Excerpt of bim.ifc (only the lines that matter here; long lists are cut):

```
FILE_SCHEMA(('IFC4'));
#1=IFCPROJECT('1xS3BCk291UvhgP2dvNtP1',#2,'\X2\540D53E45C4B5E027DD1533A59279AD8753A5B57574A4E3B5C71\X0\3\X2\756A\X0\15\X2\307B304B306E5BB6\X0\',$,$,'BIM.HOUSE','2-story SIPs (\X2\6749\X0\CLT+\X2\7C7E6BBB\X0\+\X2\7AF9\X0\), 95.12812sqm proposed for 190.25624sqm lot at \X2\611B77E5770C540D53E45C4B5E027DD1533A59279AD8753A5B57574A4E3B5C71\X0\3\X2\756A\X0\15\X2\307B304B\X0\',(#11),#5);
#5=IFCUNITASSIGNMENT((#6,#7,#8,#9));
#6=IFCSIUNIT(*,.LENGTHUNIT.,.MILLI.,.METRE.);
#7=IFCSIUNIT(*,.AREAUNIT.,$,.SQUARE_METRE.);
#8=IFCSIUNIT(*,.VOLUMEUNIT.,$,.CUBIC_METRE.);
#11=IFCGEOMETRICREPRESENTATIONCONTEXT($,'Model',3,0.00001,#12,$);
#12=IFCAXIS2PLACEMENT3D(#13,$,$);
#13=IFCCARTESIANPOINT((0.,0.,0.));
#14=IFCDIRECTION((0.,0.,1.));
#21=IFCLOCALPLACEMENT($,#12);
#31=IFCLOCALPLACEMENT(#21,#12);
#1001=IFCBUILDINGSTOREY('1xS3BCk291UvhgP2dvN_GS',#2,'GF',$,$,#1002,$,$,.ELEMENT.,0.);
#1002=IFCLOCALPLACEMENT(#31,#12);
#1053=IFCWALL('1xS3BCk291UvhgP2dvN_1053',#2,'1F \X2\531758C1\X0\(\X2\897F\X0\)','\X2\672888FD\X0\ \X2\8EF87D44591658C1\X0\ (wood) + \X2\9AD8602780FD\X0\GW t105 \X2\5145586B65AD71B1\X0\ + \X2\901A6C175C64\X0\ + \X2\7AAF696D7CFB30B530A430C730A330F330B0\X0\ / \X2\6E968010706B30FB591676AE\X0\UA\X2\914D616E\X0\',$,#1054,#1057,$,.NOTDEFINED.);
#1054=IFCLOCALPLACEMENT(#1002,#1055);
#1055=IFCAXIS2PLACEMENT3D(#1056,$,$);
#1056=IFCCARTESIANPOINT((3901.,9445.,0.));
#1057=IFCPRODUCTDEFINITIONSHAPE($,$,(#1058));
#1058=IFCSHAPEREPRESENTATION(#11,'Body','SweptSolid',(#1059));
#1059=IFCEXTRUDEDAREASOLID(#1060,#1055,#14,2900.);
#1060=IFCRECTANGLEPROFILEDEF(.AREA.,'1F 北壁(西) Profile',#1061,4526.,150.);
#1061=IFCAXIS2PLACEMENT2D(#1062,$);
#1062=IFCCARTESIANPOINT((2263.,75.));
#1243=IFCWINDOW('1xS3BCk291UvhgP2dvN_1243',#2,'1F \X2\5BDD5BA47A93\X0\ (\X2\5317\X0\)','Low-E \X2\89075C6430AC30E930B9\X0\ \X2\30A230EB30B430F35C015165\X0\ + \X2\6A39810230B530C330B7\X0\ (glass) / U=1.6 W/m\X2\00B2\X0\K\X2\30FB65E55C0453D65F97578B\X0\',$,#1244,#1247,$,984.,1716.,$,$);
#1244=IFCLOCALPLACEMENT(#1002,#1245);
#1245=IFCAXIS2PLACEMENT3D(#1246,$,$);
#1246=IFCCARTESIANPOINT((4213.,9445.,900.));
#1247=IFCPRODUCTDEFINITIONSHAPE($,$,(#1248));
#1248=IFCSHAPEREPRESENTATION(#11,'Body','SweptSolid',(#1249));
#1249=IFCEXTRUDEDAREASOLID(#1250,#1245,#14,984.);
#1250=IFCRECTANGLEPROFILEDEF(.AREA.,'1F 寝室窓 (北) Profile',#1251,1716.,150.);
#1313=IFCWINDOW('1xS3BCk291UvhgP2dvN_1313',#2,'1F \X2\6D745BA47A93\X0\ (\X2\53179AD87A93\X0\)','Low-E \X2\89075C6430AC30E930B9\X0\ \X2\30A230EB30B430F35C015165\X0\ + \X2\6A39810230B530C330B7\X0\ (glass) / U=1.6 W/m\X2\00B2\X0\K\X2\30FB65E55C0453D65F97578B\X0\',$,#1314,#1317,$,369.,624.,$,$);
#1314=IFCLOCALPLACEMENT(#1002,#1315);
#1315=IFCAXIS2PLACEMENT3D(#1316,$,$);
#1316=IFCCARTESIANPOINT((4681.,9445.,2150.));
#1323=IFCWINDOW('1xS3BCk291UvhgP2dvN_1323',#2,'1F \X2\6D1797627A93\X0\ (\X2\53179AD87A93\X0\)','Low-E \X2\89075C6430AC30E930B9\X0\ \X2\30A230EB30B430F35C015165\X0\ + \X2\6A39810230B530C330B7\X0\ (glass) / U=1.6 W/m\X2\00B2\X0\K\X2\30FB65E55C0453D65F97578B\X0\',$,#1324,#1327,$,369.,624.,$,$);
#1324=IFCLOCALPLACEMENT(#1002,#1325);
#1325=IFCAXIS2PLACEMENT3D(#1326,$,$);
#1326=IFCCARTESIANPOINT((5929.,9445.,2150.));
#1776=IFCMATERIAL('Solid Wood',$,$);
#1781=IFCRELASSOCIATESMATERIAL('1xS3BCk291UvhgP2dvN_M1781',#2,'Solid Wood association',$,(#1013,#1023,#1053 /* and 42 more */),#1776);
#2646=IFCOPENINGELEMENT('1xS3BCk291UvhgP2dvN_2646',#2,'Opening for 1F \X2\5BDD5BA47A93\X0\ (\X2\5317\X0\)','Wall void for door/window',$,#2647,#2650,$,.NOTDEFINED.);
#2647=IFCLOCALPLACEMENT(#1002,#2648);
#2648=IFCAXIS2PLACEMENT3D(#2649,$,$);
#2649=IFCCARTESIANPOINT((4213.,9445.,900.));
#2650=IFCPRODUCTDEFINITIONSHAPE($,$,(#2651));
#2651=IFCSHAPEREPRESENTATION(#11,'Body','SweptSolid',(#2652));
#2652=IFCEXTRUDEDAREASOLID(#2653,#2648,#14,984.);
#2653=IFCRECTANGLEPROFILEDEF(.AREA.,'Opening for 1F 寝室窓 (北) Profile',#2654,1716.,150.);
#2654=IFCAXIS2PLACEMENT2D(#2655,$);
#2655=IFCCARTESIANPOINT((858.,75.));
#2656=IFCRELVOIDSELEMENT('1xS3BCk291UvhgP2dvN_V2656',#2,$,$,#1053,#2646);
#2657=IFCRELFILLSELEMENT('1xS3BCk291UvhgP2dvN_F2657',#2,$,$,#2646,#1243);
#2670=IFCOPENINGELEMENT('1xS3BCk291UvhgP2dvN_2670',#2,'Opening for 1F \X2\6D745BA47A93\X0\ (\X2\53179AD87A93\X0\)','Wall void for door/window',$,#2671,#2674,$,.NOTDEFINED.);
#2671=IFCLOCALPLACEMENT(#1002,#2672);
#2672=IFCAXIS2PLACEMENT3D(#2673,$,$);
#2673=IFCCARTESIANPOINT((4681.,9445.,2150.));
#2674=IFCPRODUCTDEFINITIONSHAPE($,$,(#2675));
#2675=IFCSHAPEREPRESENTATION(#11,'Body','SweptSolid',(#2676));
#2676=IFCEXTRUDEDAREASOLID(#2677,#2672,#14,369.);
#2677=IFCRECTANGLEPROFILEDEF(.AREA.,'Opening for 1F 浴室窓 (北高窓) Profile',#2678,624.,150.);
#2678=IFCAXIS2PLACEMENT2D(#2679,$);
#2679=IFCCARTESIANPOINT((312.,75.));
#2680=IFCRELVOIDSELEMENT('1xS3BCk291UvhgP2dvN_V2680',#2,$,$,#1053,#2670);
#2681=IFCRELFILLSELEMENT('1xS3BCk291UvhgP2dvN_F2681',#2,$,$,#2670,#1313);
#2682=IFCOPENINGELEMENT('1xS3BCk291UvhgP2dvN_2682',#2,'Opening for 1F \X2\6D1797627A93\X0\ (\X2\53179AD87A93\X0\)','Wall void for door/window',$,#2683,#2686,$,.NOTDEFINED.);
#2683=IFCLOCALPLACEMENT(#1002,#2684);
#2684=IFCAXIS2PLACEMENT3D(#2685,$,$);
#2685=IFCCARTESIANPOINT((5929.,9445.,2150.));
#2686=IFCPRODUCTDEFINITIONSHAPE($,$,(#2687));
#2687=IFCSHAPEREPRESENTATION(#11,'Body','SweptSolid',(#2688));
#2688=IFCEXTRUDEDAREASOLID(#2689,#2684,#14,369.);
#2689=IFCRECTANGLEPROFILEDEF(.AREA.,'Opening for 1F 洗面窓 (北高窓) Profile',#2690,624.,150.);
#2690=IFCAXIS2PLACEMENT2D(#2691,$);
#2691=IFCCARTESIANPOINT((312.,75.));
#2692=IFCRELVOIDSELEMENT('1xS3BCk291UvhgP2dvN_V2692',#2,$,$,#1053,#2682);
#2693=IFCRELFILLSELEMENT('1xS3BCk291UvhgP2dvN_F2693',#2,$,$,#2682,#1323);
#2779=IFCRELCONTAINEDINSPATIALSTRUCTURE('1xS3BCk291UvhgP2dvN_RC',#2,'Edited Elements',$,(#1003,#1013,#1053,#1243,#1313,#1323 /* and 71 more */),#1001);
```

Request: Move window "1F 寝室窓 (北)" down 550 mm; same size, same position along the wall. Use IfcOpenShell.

```python
import numpy as np
import ifcopenshell
import ifcopenshell.api.geometry
import ifcopenshell.util.placement
import ifcopenshell.util.unit

model = ifcopenshell.open("bim.ifc")
unit_scale = ifcopenshell.util.unit.calculate_unit_scale(model)

window = model.by_guid("1xS3BCk291UvhgP2dvN_1243")
opening = window.FillsVoids[0].RelatingOpeningElement
dz = -0.55 / unit_scale

shift = np.array([0.0, 0.0, dz])
# The window is not placed relative to its opening, so move both.
for product in (opening, window):
    matrix = ifcopenshell.util.placement.get_local_placement(product.ObjectPlacement)
    matrix[:3, 3] += shift
    ifcopenshell.api.geometry.edit_object_placement(model, product=product, matrix=matrix, is_si=False)

print(f"moved by {dz * unit_scale:+.3f} m")

model.write("bim_updated.ifc")
```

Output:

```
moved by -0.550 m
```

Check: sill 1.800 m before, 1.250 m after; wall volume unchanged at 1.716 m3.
